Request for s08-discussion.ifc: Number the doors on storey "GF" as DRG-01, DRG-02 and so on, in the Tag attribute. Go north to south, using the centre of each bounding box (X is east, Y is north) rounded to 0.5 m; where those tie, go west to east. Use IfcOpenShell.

First a look at what the model holds.

```python
import ifcopenshell
import ifcopenshell.util.element
import ifcopenshell.util.placement

model = ifcopenshell.open("s08-discussion.ifc")
print(model.schema)
storey = next(s for s in model.by_type("IfcBuildingStorey") if s.Name == "GF")
doors = [e for e in ifcopenshell.util.element.get_decomposition(storey) if e.is_a("IfcDoor")]
for e in sorted(doors, key=lambda e: e.id()):
    origin = ifcopenshell.util.placement.get_local_placement(e.ObjectPlacement)[:3, 3]
    print(e.id(), e.Tag, e.Name, origin.round(2) + 0.0, sep=" | ")
```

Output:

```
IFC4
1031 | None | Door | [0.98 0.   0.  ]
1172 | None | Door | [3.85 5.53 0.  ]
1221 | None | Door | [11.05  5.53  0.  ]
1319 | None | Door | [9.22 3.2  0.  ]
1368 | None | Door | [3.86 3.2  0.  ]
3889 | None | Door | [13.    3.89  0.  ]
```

```python
import ifcopenshell
import ifcopenshell.geom
import ifcopenshell.util.element
import ifcopenshell.util.shape

model = ifcopenshell.open("s08-discussion.ifc")
settings = ifcopenshell.geom.settings()
settings.set("use-world-coords", True)


def centre(element):
    shape = ifcopenshell.geom.create_shape(settings, element)
    return ifcopenshell.util.shape.get_bbox_centroid(shape.geometry)


storey = next(s for s in model.by_type("IfcBuildingStorey") if s.Name == "GF")
doors = [e for e in ifcopenshell.util.element.get_decomposition(storey) if e.is_a("IfcDoor")]

# Insertion points can sit at a corner or the storey origin, so sort by the geometry (in metres).
centres = {e: centre(e) for e in doors}
doors.sort(key=lambda e: (-round(centres[e][1] / 0.5), centres[e][0]))

for i, e in enumerate(doors, start=1):
    number = f"DRG-{i:02d}"
    e.Tag = number
    print(e.id(), number)

model.write("s08-discussion_edited.ifc")
```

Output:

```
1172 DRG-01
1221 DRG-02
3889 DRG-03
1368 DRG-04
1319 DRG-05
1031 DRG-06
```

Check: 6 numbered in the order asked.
